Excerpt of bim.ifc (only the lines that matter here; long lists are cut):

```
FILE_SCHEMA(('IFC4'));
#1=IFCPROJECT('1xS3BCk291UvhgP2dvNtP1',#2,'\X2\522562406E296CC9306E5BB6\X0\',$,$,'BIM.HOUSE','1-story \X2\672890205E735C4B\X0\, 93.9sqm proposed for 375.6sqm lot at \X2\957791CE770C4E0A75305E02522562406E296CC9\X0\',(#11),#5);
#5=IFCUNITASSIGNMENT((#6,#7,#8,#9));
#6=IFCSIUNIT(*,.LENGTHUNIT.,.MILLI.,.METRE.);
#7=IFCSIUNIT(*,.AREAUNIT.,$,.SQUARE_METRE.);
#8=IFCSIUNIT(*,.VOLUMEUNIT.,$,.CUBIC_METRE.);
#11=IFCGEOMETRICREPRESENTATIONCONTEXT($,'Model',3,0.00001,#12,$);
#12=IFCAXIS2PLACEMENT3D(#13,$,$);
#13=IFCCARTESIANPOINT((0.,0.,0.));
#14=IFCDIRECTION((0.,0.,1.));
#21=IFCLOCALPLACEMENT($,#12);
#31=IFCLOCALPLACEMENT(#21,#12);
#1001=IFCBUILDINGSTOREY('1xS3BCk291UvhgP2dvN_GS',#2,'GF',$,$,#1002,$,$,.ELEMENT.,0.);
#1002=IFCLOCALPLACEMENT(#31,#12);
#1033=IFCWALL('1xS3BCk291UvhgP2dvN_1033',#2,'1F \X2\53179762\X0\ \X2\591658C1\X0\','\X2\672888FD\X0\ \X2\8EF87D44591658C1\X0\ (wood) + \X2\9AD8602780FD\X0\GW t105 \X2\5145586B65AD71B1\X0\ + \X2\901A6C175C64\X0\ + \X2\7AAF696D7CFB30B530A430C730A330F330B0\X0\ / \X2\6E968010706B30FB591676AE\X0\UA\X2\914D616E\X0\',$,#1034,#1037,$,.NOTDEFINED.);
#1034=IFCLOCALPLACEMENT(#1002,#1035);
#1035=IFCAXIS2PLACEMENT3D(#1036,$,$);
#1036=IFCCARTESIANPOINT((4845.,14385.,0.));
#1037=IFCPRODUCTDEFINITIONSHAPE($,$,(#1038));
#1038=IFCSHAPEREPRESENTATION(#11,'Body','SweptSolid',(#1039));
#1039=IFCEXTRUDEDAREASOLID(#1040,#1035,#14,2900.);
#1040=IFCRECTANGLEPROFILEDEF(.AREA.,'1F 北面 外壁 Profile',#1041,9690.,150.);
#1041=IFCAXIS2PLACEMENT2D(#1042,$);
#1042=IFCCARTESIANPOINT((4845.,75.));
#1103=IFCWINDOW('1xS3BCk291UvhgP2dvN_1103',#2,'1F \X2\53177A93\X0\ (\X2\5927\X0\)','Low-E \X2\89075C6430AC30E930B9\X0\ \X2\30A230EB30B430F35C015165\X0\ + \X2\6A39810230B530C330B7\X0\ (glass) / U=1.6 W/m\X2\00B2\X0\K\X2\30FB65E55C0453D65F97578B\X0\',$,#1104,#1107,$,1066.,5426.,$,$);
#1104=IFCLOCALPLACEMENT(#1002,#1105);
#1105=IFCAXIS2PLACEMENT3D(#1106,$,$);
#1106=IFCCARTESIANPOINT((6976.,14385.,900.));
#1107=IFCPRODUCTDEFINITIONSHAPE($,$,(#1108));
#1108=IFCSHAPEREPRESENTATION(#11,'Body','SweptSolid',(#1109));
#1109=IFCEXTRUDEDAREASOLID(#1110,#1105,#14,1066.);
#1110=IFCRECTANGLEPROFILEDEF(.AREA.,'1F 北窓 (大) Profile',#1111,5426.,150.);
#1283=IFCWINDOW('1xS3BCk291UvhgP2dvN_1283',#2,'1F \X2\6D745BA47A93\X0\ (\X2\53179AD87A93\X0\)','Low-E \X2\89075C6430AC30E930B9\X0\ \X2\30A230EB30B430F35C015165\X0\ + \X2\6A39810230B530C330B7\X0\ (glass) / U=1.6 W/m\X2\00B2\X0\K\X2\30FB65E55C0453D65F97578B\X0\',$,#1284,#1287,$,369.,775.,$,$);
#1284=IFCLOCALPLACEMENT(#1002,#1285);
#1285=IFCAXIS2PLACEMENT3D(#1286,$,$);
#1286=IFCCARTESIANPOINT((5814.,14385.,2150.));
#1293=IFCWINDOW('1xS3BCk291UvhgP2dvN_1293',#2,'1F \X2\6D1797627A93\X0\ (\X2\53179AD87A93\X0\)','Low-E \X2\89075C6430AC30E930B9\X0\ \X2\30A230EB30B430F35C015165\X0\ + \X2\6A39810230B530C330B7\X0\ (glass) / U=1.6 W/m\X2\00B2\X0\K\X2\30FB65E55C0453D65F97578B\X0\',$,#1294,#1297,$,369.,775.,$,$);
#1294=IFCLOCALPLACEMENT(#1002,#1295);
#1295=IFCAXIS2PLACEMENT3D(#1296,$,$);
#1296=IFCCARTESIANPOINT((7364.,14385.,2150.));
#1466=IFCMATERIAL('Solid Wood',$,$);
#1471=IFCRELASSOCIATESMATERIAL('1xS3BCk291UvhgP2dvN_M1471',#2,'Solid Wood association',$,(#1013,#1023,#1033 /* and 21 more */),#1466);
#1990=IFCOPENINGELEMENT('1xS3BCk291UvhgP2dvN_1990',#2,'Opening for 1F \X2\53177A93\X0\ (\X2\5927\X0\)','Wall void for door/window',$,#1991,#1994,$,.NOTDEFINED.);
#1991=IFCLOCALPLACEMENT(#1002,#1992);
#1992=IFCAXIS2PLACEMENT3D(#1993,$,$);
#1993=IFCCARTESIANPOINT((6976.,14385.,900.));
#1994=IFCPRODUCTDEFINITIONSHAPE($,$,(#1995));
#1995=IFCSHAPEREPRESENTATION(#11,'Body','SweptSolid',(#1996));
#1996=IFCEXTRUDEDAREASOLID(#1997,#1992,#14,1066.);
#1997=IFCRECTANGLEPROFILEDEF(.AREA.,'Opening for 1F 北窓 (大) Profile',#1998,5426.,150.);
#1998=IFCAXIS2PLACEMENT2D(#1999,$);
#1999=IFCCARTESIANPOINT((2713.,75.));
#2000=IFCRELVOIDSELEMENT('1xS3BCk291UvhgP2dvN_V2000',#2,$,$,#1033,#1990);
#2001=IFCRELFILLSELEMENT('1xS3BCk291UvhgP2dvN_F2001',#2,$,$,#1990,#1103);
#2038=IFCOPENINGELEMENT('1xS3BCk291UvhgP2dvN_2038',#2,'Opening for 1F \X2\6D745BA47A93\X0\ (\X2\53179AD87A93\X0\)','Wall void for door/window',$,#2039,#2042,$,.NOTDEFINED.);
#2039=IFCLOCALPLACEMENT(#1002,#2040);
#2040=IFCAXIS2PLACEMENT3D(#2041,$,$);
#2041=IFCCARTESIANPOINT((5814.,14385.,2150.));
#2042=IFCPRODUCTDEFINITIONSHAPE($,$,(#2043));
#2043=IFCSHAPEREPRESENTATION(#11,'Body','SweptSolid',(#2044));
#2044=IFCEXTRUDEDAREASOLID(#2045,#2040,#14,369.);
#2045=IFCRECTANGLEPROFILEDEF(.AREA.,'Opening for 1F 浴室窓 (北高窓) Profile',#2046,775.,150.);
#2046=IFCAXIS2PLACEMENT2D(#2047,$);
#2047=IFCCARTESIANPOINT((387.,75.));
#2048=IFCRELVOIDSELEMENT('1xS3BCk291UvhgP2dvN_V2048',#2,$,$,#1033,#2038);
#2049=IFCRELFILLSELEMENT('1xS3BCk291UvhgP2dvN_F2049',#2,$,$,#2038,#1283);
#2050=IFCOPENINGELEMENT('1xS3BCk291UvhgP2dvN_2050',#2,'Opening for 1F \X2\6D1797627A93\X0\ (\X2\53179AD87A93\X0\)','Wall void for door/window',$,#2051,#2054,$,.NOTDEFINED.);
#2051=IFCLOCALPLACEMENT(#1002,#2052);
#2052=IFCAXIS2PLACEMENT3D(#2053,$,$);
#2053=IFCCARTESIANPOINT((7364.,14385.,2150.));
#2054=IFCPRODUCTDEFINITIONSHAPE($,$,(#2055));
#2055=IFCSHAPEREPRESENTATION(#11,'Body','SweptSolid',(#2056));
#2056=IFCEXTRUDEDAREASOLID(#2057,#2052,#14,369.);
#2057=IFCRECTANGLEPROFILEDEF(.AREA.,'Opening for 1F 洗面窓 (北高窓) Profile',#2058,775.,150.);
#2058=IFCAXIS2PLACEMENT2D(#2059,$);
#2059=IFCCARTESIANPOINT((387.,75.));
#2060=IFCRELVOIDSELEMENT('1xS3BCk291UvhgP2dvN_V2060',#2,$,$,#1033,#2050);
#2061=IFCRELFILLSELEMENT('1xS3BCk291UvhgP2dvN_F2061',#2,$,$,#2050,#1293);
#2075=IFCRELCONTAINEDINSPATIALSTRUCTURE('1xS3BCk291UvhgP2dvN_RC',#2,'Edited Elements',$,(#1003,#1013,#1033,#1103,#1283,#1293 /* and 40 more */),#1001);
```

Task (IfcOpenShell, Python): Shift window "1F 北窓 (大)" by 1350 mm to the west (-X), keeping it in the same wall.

```python
import ifcopenshell
import ifcopenshell.api.geometry
import ifcopenshell.util.placement

model = ifcopenshell.open("bim.ifc")

window = model.by_guid("1xS3BCk291UvhgP2dvN_1103")
opening = window.FillsVoids[0].RelatingOpeningElement
wall = opening.VoidsElements[0].RelatingBuildingElement

wall_matrix = ifcopenshell.util.placement.get_local_placement(wall.ObjectPlacement)
shift = wall_matrix[:3, 0] * -1350.0
before = ifcopenshell.util.placement.get_local_placement(window.ObjectPlacement)[:3, 3].copy()

# The window is not placed relative to its opening, so move both.
for product in (opening, window):
    matrix = ifcopenshell.util.placement.get_local_placement(product.ObjectPlacement)
    matrix[:3, 3] += shift
    ifcopenshell.api.geometry.edit_object_placement(model, product=product, matrix=matrix, is_si=False)

after = ifcopenshell.util.placement.get_local_placement(window.ObjectPlacement)[:3, 3]
print("window moved by", (after - before).round(3) + 0.0)

model.write("bim_updated.ifc")
```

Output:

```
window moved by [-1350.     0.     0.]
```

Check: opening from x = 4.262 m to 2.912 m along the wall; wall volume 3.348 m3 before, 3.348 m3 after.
